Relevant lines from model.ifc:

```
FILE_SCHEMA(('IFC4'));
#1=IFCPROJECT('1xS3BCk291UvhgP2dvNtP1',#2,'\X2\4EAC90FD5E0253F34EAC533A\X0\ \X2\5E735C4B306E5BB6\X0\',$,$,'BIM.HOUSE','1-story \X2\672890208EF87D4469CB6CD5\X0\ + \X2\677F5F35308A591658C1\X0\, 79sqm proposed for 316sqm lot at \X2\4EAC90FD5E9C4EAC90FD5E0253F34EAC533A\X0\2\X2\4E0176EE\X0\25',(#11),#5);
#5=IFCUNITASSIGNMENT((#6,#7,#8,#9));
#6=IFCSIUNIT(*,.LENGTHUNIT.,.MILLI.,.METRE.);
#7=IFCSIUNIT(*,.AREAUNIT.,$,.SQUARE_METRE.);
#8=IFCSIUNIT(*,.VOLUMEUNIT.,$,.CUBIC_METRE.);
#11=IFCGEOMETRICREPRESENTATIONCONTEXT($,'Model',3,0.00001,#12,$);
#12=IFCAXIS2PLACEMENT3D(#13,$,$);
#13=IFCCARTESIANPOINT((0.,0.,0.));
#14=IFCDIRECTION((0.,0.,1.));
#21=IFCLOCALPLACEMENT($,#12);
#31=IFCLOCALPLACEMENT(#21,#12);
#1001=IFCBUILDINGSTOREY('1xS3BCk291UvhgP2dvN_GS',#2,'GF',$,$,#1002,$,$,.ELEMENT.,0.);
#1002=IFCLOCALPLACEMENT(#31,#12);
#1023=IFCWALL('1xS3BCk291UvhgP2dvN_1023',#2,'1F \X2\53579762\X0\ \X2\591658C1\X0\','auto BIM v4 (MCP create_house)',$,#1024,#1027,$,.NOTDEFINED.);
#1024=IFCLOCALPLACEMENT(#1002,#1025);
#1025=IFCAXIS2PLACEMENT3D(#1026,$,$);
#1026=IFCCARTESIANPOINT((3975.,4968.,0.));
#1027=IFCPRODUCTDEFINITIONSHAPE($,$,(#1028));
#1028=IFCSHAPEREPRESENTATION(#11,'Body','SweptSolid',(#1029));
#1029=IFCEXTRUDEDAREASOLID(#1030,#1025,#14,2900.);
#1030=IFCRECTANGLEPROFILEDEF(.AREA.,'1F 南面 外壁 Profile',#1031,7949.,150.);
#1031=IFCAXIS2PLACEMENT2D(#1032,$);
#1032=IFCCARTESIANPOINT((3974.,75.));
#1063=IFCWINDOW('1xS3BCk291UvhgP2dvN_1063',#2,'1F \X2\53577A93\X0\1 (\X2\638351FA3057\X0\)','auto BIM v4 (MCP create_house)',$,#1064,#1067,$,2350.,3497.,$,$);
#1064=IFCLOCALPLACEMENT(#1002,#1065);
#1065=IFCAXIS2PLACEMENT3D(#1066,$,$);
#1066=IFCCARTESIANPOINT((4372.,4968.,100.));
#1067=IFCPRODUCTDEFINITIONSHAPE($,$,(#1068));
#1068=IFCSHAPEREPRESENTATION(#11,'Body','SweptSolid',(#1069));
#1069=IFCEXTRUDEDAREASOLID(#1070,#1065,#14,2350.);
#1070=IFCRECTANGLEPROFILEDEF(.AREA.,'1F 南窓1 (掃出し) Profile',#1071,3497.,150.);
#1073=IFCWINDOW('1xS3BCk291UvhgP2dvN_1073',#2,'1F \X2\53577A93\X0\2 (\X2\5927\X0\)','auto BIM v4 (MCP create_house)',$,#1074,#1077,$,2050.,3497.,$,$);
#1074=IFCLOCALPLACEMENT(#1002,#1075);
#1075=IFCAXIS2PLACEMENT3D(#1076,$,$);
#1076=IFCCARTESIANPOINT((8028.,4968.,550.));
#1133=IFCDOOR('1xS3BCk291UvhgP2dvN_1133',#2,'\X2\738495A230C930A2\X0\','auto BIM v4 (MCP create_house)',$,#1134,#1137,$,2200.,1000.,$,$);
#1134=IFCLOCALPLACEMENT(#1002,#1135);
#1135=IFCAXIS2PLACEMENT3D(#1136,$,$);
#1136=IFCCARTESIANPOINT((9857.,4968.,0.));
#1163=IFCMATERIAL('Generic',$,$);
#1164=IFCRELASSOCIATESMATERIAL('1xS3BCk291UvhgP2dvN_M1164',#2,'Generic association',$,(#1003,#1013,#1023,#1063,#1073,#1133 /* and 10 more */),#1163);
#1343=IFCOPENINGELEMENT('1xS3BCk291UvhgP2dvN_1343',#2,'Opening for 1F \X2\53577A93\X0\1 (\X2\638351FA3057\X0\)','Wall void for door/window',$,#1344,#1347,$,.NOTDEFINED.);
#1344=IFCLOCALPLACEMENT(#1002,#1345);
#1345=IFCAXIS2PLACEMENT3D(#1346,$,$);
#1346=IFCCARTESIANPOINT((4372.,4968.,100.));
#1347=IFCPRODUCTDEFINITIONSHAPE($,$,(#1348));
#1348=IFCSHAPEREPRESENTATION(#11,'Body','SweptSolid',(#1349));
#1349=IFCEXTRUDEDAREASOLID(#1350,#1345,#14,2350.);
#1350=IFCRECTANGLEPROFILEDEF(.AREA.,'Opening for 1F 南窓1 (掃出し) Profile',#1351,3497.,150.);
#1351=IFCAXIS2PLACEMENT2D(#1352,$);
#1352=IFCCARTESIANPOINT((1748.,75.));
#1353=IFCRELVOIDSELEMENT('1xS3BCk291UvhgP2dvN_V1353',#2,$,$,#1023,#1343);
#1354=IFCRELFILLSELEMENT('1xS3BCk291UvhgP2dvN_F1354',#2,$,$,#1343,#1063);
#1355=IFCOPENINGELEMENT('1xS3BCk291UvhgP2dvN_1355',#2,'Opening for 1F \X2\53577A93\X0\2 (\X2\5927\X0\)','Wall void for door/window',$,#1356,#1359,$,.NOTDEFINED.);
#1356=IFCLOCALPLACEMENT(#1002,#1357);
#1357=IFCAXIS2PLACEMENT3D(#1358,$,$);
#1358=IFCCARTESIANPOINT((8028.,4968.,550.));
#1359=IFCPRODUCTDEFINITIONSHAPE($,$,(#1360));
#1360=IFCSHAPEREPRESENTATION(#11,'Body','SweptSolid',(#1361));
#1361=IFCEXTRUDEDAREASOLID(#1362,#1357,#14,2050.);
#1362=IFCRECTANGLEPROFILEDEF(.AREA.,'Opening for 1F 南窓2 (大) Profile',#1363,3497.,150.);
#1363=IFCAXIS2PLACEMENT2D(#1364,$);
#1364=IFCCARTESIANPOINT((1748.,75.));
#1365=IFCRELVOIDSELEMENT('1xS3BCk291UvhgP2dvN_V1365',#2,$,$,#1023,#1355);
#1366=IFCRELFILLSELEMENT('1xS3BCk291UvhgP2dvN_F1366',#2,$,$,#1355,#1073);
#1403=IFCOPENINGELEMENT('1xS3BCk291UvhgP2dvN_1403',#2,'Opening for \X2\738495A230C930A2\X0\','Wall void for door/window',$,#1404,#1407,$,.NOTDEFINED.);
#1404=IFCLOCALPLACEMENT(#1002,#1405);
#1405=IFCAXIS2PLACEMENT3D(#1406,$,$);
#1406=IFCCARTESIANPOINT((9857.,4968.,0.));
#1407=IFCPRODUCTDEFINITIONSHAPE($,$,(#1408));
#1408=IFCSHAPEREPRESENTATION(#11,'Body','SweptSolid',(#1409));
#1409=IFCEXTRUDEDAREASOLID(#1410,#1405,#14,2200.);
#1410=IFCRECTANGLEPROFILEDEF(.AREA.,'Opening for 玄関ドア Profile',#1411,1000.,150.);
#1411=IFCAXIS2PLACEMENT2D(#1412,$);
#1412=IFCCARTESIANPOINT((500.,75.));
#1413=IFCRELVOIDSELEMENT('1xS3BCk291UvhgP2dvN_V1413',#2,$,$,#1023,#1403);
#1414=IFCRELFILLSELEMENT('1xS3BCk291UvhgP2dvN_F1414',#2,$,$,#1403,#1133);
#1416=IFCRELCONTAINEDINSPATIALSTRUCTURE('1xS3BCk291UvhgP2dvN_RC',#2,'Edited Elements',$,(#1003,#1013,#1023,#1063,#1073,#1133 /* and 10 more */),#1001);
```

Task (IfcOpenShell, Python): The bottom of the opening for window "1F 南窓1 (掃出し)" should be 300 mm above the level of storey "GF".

```python
import numpy as np
import ifcopenshell
import ifcopenshell.api.geometry
import ifcopenshell.geom
import ifcopenshell.util.element
import ifcopenshell.util.placement
import ifcopenshell.util.shape
import ifcopenshell.util.unit

model = ifcopenshell.open("model.ifc")
unit_scale = ifcopenshell.util.unit.calculate_unit_scale(model)

window = model.by_guid("1xS3BCk291UvhgP2dvN_1063")
opening = window.FillsVoids[0].RelatingOpeningElement
storey = ifcopenshell.util.element.get_container(window, ifc_class="IfcBuildingStorey")
level = ifcopenshell.util.placement.get_local_placement(storey.ObjectPlacement)[2, 3]

# The opening's origin need not be at the sill, so measure its lowest point.
shape = ifcopenshell.geom.create_shape(ifcopenshell.geom.settings(), opening)
bottom = ifcopenshell.util.shape.get_shape_bottom_elevation(shape, shape.geometry) / unit_scale
dz = level + 300.0 - bottom

shift = np.array([0.0, 0.0, dz])
# The window is not placed relative to its opening, so move both.
for product in (opening, window):
    matrix = ifcopenshell.util.placement.get_local_placement(product.ObjectPlacement)
    matrix[:3, 3] += shift
    ifcopenshell.api.geometry.edit_object_placement(model, product=product, matrix=matrix, is_si=False)

print(f"moved by {dz * unit_scale:+.3f} m")

model.write("model_rev.ifc")
```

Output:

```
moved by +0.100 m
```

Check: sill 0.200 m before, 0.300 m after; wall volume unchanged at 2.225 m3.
